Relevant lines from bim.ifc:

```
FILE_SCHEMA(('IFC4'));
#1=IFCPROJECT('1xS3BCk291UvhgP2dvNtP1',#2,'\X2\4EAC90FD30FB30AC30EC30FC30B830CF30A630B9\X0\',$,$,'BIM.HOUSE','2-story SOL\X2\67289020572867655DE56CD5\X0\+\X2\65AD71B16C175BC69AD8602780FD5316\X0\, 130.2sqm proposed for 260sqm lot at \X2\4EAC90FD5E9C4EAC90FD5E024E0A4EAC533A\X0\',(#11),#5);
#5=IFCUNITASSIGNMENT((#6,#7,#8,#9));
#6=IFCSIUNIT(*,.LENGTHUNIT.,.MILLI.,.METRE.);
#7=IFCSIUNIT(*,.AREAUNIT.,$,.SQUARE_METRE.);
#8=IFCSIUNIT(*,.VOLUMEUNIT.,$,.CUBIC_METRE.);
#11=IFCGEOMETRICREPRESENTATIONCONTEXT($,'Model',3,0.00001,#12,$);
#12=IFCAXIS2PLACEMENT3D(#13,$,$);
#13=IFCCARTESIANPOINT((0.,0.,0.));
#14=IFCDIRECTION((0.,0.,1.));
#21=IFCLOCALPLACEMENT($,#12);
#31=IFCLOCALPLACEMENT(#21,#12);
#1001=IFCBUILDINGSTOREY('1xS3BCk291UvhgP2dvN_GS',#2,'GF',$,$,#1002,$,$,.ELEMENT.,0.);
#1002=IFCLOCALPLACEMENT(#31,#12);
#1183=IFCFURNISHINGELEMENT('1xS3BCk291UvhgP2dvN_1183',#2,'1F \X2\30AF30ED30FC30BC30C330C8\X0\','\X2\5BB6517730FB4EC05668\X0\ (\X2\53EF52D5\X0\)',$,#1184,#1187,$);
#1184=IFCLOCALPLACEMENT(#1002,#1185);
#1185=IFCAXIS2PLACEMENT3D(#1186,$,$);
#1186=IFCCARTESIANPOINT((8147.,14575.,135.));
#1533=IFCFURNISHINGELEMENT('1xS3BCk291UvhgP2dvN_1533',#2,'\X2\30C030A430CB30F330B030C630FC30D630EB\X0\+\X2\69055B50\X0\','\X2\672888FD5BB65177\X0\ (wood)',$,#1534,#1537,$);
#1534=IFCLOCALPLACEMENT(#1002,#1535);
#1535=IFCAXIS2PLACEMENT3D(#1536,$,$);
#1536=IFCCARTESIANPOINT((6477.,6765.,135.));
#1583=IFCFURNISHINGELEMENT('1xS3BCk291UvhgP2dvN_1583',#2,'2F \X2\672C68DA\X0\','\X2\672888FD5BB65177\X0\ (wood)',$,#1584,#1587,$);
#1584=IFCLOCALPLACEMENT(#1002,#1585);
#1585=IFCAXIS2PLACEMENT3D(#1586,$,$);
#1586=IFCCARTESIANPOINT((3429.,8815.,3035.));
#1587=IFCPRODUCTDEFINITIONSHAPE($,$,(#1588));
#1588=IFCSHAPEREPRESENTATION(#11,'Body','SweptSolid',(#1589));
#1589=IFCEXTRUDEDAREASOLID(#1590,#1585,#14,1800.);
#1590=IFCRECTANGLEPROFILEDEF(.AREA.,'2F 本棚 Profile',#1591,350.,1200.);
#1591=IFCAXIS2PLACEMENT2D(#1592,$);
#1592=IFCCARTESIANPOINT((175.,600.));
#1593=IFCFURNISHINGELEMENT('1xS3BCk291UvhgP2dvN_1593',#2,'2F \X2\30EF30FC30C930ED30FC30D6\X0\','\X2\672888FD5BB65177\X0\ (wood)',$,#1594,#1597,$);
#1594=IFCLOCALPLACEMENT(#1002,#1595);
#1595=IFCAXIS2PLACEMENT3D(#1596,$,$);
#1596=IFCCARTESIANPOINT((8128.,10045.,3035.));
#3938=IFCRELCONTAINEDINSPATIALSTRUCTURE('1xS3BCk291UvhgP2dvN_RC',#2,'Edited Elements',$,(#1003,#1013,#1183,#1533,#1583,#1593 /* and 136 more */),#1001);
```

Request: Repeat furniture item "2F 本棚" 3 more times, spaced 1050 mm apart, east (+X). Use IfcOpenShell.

```python
import numpy as np
import ifcopenshell
import ifcopenshell.api.geometry
import ifcopenshell.api.root
import ifcopenshell.util.element
import ifcopenshell.util.placement
import ifcopenshell.util.unit

model = ifcopenshell.open("bim.ifc")
unit_scale = ifcopenshell.util.unit.calculate_unit_scale(model)


def reuse_history(source, copy):
    """copy_class also copies each property set's owner history, people and application; keep the originals."""
    for rel in copy.IsDefinedBy:
        if rel.is_a("IfcRelDefinesByProperties") and (history := rel.RelatingPropertyDefinition.OwnerHistory):
            rel.RelatingPropertyDefinition.OwnerHistory = source.OwnerHistory
            ifcopenshell.util.element.remove_deep2(model, history)


source = model.by_guid("1xS3BCk291UvhgP2dvN_1583")
base = ifcopenshell.util.placement.get_local_placement(source.ObjectPlacement)
step = np.array([1.0, 0.0, 0.0]) * 1.05 / unit_scale

for i in range(1, 4):
    copy = ifcopenshell.api.root.copy_class(model, product=source)
    copy.Representation = ifcopenshell.util.element.copy_deep(
        model, source.Representation, exclude=["IfcGeometricRepresentationContext", "IfcRepresentationMap"]
    )
    reuse_history(source, copy)
    matrix = base.copy()
    matrix[:3, 3] += i * step
    print("added at", matrix[:3, 3].round(3) + 0.0)
    ifcopenshell.api.geometry.edit_object_placement(model, product=copy, matrix=matrix, is_si=False)

model.write("bim_updated.ifc")
```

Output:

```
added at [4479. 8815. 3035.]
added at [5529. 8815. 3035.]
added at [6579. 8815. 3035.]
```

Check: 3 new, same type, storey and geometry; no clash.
